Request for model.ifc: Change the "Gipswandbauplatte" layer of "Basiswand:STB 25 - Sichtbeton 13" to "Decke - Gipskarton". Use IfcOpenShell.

First a look at what the model holds.

```python
import ifcopenshell
import ifcopenshell.util.element

model = ifcopenshell.open("model.ifc")
print(model.schema)
for layer_set in model.by_type("IfcMaterialLayerSet"):
    if layer_set.LayerSetName == "Basiswand:STB 25 - Sichtbeton 13":
        for layer in layer_set.MaterialLayers:
            print(layer.id(), layer.Material and layer.Material.Name, layer.LayerThickness, sep=" | ")
        print(len(ifcopenshell.util.element.get_elements_by_material(model, layer_set)), "elements and types use it")
print(sorted(m.Name for m in model.by_type("IfcMaterial") if m.Name)[:60])
```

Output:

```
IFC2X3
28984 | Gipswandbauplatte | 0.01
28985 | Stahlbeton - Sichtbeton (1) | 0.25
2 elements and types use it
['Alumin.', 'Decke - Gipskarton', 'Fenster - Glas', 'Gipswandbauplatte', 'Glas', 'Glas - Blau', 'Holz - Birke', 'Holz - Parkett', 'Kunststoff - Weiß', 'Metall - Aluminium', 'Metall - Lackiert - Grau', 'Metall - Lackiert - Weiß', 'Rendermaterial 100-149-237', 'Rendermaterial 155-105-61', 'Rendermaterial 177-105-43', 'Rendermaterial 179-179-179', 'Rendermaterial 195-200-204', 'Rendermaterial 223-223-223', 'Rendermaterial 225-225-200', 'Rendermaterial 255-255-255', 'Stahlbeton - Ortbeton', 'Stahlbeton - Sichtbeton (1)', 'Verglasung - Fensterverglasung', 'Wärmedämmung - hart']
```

```python
import ifcopenshell
import ifcopenshell.api.material

model = ifcopenshell.open("model.ifc")

layer_set = next(s for s in model.by_type("IfcMaterialLayerSet") if s.LayerSetName == "Basiswand:STB 25 - Sichtbeton 13")
layer = next(l for l in layer_set.MaterialLayers if l.Material and l.Material.Name == "Gipswandbauplatte")
material = next(m for m in model.by_type("IfcMaterial") if m.Name == "Decke - Gipskarton")

# Point this one layer at the other material; renaming the old one would change it everywhere.
ifcopenshell.api.material.edit_layer(model, layer=layer, attributes={}, material=material)

print([l.Material.Name if l.Material else None for l in layer_set.MaterialLayers])

model.write("model_edited.ifc")
```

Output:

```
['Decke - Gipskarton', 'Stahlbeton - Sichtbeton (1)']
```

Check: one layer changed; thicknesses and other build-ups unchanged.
